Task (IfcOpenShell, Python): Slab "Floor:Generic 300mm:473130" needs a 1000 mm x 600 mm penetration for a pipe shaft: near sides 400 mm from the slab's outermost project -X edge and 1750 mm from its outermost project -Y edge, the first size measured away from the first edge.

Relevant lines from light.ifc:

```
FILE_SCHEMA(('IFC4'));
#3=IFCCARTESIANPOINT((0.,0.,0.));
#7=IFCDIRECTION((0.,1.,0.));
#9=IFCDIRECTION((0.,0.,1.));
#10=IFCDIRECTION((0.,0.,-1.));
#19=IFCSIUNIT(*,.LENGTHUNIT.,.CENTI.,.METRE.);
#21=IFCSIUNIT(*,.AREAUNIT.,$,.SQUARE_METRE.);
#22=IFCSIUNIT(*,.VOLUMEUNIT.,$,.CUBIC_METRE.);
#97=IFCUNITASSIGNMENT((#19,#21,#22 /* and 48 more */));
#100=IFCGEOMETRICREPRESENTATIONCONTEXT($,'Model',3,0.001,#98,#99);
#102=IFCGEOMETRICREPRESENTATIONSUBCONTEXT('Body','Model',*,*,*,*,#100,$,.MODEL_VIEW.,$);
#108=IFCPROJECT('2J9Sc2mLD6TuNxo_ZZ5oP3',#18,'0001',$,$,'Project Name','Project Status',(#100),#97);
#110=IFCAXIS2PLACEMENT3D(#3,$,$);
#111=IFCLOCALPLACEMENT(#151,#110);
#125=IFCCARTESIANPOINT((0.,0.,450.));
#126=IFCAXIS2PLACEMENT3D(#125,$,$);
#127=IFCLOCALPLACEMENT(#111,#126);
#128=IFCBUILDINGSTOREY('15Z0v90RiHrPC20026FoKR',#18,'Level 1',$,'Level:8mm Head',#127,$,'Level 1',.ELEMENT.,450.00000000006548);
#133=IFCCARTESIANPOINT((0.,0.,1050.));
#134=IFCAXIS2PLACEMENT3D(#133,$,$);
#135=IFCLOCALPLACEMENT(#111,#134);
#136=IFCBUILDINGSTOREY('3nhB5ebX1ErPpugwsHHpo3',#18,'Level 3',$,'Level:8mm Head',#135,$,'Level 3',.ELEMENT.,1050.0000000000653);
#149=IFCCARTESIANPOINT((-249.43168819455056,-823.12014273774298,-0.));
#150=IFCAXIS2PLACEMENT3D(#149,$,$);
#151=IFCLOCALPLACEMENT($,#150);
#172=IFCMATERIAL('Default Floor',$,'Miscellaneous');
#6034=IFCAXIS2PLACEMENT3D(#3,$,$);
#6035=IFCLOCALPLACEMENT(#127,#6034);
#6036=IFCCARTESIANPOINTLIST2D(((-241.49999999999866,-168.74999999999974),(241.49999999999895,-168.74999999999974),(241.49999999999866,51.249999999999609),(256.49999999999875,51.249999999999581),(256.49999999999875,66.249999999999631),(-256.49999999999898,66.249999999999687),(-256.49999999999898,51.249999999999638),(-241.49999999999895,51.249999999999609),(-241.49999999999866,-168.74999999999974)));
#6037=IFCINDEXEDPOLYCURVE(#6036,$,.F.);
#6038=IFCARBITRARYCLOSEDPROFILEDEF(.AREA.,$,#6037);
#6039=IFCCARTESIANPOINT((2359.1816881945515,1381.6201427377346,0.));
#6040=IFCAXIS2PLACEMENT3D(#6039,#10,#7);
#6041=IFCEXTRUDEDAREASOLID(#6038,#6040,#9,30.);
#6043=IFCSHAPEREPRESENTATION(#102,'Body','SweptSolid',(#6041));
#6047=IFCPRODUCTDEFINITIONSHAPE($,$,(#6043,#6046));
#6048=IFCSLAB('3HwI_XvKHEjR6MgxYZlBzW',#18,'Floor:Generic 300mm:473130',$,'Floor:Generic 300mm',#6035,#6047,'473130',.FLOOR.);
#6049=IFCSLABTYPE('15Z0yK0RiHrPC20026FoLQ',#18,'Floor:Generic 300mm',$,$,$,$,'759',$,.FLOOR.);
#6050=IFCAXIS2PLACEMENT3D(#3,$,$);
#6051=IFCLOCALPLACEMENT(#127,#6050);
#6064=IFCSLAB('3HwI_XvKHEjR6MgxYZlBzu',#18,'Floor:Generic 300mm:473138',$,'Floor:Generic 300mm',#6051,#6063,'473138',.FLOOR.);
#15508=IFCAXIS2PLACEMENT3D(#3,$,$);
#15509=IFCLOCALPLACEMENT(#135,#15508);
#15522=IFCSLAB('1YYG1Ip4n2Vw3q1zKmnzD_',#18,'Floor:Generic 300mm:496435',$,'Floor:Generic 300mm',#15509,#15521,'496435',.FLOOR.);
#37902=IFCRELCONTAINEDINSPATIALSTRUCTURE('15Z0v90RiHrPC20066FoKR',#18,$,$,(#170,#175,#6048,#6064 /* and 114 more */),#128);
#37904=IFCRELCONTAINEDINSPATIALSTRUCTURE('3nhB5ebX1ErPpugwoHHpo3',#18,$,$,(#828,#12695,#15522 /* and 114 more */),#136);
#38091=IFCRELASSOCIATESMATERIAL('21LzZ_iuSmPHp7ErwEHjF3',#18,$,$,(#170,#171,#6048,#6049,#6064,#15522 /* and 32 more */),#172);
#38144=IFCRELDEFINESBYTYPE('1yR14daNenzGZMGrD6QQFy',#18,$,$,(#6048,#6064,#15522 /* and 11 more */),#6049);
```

```python
import numpy as np
import ifcopenshell
import ifcopenshell.api.feature
import ifcopenshell.api.geometry
import ifcopenshell.api.root
import ifcopenshell.geom
import ifcopenshell.util.placement
import ifcopenshell.util.representation
import ifcopenshell.util.shape
import ifcopenshell.util.unit

model = ifcopenshell.open("light.ifc")
unit_scale = ifcopenshell.util.unit.calculate_unit_scale(model)
settings = ifcopenshell.geom.settings()


def volume(element):
    """Net volume in cubic metres, openings subtracted."""
    shape = ifcopenshell.geom.create_shape(settings, element)
    return ifcopenshell.util.shape.get_volume(shape.geometry)


slab = model.by_guid("3HwI_XvKHEjR6MgxYZlBzW")
before = volume(slab)

# Extent in the slab's own axes, in metres. The edges named are its -X and -Y sides.
slab_shape = ifcopenshell.geom.create_shape(settings, slab)
vertices = ifcopenshell.util.shape.get_vertices(slab_shape.geometry)
x_min, y_min, bottom = vertices.min(axis=0)
top = vertices[:, 2].max()

opening = ifcopenshell.api.root.create_entity(model, ifc_class="IfcOpeningElement", name="Pipe shaft opening", predefined_type="OPENING")
context = ifcopenshell.util.representation.get_context(model, "Model", "Body", "MODEL_VIEW")
width, depth = 1, 0.6
outline = [(0.0, 0.0), (width, 0.0), (width, depth), (0.0, depth), (0.0, 0.0)]
# Overshoot both faces by 50 mm so the cut is clean.
shape = ifcopenshell.api.geometry.add_slab_representation(
    model, context=context, depth=top - bottom + 0.1, polyline=outline
)
ifcopenshell.api.geometry.assign_representation(model, product=opening, representation=shape)

matrix = ifcopenshell.util.placement.get_local_placement(slab.ObjectPlacement)
matrix[:, 3] = matrix @ np.append(np.array([x_min + 0.4, y_min + 1.75, bottom - 0.05]) / unit_scale, 1.0)
ifcopenshell.api.geometry.edit_object_placement(model, product=opening, matrix=matrix, is_si=False)
ifcopenshell.api.feature.add_feature(model, feature=opening, element=slab)

after = volume(slab)

print(f"slab volume {before:.3f} -> {after:.3f} m3")

model.write("light_edited.ifc")
```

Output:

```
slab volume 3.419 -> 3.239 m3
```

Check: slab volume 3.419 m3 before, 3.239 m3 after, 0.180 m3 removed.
